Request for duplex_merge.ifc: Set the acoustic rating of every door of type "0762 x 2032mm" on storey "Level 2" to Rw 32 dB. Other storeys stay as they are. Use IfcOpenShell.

First a look at what the model holds.

```python
import ifcopenshell
import ifcopenshell.util.element

model = ifcopenshell.open("duplex_merge.ifc")
print(model.schema)
storey = next(s for s in model.by_type("IfcBuildingStorey") if s.Name == "Level 2")
doors = [e for e in ifcopenshell.util.element.get_decomposition(storey) if e.is_a("IfcDoor")]
seen = {}
for e in doors:
    element_type = ifcopenshell.util.element.get_type(e)
    key = (element_type.Name if element_type != e and element_type else None, ifcopenshell.util.element.get_pset(e, "Pset_DoorCommon", "AcousticRating"))
    seen[key] = seen.get(key, 0) + 1
for (name, value), count in sorted(seen.items(), key=str):
    print(count, "x", name, "|", value)
```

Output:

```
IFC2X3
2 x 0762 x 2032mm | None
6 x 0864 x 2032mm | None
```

```python
import ifcopenshell
import ifcopenshell.api.pset
import ifcopenshell.util.element

model = ifcopenshell.open("duplex_merge.ifc")

storey = next(s for s in model.by_type("IfcBuildingStorey") if s.Name == "Level 2")
doors = [e for e in ifcopenshell.util.element.get_decomposition(storey) if e.is_a("IfcDoor")]

count = 0
for e in doors:
    element_type = ifcopenshell.util.element.get_type(e)
    if element_type in (None, e) or element_type.Name != "0762 x 2032mm":
        continue
    # add_pset returns the element's existing set when there is one.
    pset = ifcopenshell.api.pset.add_pset(model, product=e, name="Pset_DoorCommon")
    ifcopenshell.api.pset.edit_pset(model, pset=pset, properties={"AcousticRating": "Rw 32 dB"})
    count += 1

print(count, "doors updated")

model.write("duplex_merge_v2.ifc")
```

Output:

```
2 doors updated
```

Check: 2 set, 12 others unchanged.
